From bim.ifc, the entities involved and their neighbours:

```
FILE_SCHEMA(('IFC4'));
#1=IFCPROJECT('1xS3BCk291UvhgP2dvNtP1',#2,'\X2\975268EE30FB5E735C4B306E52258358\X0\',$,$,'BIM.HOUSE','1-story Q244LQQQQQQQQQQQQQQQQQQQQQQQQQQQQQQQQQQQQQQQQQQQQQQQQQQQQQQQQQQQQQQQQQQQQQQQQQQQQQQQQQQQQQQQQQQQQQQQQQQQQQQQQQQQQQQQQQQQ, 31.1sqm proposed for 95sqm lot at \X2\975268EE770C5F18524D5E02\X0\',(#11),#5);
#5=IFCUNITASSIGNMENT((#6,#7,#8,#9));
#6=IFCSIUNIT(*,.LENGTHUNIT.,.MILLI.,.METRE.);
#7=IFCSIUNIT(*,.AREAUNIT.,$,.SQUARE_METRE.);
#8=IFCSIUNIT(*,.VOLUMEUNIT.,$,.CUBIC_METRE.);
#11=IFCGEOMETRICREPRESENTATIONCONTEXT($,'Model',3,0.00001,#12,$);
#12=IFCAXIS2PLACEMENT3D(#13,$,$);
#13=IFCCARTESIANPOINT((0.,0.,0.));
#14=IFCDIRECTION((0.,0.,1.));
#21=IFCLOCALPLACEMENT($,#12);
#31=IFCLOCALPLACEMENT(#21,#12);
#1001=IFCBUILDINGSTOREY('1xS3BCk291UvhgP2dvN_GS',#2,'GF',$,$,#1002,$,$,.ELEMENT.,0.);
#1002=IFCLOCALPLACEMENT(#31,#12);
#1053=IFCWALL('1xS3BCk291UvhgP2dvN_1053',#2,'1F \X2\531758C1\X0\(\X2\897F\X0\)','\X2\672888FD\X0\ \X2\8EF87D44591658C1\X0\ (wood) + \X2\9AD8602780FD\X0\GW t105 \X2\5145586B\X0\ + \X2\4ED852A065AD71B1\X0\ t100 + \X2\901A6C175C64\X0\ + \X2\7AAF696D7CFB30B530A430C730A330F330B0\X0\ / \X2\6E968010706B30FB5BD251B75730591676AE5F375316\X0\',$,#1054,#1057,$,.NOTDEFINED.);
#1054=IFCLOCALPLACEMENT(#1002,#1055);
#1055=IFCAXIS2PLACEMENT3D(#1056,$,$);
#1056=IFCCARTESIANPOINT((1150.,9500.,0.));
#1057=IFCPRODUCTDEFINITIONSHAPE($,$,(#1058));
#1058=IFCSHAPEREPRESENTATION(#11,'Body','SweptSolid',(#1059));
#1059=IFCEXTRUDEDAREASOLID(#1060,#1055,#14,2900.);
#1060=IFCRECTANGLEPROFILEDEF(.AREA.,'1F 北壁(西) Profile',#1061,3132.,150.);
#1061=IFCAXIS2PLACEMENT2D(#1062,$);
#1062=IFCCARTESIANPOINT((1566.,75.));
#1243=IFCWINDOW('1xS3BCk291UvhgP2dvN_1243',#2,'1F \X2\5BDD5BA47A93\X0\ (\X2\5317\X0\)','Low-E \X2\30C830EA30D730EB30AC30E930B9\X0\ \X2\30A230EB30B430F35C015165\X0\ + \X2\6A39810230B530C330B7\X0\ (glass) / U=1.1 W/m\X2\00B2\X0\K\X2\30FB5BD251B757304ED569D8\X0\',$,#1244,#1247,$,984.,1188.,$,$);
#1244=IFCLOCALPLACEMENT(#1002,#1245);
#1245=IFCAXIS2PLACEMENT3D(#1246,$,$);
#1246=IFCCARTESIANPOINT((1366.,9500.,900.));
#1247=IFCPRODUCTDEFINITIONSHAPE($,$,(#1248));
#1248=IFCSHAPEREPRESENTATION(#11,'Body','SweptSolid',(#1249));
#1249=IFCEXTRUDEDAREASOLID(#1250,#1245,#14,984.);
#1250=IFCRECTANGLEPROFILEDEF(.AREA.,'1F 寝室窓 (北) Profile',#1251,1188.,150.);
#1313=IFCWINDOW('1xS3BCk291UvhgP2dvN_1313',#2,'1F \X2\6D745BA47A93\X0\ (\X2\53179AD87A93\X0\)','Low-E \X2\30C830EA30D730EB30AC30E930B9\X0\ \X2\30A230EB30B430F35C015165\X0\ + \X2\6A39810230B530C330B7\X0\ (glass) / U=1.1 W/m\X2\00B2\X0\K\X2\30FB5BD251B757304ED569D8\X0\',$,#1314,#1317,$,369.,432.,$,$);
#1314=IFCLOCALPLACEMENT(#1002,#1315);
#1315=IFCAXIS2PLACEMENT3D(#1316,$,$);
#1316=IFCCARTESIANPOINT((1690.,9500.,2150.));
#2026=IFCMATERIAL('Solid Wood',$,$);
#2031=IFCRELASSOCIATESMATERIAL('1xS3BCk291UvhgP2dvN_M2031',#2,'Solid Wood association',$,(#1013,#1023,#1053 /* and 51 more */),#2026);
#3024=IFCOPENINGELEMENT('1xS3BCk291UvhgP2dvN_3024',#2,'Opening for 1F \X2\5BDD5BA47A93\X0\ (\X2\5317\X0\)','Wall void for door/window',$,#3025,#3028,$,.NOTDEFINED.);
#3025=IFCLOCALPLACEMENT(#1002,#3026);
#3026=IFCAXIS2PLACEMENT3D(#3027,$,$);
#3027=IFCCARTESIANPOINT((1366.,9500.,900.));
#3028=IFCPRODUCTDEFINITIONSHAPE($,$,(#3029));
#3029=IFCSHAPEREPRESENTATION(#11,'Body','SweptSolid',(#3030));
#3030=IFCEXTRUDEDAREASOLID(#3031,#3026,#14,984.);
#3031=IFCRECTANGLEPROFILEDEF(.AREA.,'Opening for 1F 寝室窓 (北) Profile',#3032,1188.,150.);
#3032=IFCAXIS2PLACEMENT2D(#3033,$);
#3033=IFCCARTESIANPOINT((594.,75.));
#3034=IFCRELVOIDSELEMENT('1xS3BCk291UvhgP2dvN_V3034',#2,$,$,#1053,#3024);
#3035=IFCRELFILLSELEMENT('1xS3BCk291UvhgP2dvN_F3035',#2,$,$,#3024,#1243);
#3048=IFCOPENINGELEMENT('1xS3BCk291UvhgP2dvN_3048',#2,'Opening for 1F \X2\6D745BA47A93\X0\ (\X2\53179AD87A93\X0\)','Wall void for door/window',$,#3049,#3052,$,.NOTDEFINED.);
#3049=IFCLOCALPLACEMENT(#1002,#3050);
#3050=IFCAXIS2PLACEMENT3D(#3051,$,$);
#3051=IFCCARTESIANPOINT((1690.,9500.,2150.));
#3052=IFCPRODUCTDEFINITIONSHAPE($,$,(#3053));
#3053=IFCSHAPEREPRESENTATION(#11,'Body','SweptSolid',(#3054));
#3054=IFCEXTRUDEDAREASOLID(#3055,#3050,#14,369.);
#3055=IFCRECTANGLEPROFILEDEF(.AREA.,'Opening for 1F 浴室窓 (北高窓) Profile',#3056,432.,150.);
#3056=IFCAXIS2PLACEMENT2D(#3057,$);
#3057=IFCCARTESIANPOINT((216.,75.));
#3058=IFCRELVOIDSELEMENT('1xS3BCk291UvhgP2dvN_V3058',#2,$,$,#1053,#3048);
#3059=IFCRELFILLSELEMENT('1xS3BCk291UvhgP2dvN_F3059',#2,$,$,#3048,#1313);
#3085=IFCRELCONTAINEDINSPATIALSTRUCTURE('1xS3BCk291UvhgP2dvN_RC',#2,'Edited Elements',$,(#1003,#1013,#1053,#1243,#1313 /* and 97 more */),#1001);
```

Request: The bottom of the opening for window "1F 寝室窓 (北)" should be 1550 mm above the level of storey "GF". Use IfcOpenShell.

```python
import numpy as np
import ifcopenshell
import ifcopenshell.api.geometry
import ifcopenshell.geom
import ifcopenshell.util.element
import ifcopenshell.util.placement
import ifcopenshell.util.shape
import ifcopenshell.util.unit

model = ifcopenshell.open("bim.ifc")
unit_scale = ifcopenshell.util.unit.calculate_unit_scale(model)

window = model.by_id(1243)
opening = window.FillsVoids[0].RelatingOpeningElement
storey = ifcopenshell.util.element.get_container(window, ifc_class="IfcBuildingStorey")
level = ifcopenshell.util.placement.get_local_placement(storey.ObjectPlacement)[2, 3]

# The opening's origin need not be at the sill, so measure its lowest point.
shape = ifcopenshell.geom.create_shape(ifcopenshell.geom.settings(), opening)
bottom = ifcopenshell.util.shape.get_shape_bottom_elevation(shape, shape.geometry) / unit_scale
dz = level + 1550.0 - bottom

shift = np.array([0.0, 0.0, dz])
# The window is not placed relative to its opening, so move both.
for product in (opening, window):
    matrix = ifcopenshell.util.placement.get_local_placement(product.ObjectPlacement)
    matrix[:3, 3] += shift
    ifcopenshell.api.geometry.edit_object_placement(model, product=product, matrix=matrix, is_si=False)

print(f"moved by {dz * unit_scale:+.3f} m")

model.write("bim-out.ifc")
```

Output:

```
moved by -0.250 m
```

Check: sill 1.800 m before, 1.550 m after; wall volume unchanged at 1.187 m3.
